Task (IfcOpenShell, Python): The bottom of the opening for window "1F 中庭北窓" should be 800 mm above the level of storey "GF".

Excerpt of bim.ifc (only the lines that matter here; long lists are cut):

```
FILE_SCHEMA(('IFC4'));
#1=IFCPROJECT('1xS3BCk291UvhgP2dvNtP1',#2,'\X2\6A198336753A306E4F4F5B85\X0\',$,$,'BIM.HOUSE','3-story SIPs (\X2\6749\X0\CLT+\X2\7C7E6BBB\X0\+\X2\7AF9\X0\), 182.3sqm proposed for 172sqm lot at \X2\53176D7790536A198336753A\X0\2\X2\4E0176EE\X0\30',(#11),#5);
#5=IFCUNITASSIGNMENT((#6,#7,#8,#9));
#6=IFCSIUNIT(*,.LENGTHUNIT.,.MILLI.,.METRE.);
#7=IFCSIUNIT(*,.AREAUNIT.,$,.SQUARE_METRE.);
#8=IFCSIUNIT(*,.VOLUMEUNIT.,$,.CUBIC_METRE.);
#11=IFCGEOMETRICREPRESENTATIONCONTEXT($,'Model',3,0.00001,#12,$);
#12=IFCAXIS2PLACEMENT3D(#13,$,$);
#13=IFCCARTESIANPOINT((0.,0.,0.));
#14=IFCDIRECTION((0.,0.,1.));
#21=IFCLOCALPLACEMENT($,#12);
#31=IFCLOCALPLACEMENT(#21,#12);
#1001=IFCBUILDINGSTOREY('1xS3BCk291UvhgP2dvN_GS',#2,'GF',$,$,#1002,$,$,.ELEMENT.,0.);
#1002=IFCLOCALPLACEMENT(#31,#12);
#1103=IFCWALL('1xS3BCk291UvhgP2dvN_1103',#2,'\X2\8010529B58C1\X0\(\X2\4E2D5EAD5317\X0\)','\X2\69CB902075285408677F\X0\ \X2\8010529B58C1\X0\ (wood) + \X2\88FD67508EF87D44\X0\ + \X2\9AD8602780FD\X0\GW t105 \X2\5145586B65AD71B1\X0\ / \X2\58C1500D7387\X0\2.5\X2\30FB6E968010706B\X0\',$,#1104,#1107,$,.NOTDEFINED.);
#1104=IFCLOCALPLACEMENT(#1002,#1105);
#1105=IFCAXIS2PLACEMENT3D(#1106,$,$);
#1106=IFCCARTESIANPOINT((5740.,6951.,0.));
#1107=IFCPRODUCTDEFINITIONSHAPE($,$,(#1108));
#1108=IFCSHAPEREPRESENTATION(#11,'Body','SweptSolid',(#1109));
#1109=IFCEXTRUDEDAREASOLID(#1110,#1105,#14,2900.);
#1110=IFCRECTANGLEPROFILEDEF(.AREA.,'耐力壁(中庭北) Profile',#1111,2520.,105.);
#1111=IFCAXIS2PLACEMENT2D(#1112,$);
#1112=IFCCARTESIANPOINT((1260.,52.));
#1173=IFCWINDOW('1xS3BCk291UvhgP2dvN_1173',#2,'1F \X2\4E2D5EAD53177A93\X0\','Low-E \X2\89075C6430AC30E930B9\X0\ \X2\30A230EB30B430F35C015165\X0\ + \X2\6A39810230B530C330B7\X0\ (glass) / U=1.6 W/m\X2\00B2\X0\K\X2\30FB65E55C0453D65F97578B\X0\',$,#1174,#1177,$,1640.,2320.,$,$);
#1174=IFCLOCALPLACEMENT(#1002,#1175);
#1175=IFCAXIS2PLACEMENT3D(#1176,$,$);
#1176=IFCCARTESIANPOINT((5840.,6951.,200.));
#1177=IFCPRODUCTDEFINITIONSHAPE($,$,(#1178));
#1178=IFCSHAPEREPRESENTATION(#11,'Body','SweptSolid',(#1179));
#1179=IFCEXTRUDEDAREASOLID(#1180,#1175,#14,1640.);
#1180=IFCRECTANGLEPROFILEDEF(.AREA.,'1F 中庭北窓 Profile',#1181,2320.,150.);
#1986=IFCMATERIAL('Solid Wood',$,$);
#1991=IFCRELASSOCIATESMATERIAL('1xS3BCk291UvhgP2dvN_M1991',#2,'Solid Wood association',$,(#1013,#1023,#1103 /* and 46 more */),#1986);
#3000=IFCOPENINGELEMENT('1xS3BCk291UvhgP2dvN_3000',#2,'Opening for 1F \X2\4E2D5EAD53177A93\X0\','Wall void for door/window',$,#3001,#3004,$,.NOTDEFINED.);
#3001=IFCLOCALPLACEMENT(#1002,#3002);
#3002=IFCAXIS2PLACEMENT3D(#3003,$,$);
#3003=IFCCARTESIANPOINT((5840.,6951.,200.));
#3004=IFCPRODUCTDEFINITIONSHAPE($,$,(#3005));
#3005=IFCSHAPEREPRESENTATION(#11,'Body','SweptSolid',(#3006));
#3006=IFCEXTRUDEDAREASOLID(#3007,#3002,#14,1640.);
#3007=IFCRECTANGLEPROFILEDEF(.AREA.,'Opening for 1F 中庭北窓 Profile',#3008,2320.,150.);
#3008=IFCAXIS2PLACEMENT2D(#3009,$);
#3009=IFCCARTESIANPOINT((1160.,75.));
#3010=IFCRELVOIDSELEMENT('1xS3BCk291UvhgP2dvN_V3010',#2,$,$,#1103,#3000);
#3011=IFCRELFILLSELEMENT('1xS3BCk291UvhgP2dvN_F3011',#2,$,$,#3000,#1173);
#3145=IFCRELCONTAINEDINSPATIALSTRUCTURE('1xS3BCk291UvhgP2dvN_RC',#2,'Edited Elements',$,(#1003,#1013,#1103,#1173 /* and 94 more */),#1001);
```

```python
import numpy as np
import ifcopenshell
import ifcopenshell.api.geometry
import ifcopenshell.geom
import ifcopenshell.util.element
import ifcopenshell.util.placement
import ifcopenshell.util.shape
import ifcopenshell.util.unit

model = ifcopenshell.open("bim.ifc")
unit_scale = ifcopenshell.util.unit.calculate_unit_scale(model)

window = model.by_guid("1xS3BCk291UvhgP2dvN_1173")
opening = window.FillsVoids[0].RelatingOpeningElement
storey = ifcopenshell.util.element.get_container(window, ifc_class="IfcBuildingStorey")
level = ifcopenshell.util.placement.get_local_placement(storey.ObjectPlacement)[2, 3]

# The opening's origin need not be at the sill, so measure its lowest point.
shape = ifcopenshell.geom.create_shape(ifcopenshell.geom.settings(), opening)
bottom = ifcopenshell.util.shape.get_shape_bottom_elevation(shape, shape.geometry) / unit_scale
dz = level + 800.0 - bottom

shift = np.array([0.0, 0.0, dz])
# The window is not placed relative to its opening, so move both.
for product in (opening, window):
    matrix = ifcopenshell.util.placement.get_local_placement(product.ObjectPlacement)
    matrix[:3, 3] += shift
    ifcopenshell.api.geometry.edit_object_placement(model, product=product, matrix=matrix, is_si=False)

print(f"moved by {dz * unit_scale:+.3f} m")

model.write("bim-out.ifc")
```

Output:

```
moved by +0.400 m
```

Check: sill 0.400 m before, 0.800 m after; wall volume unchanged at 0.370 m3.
